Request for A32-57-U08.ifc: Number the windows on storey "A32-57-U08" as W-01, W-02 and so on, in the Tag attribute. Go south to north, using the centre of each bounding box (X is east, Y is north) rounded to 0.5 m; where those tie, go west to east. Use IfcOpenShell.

First a look at what the model holds.

```python
import ifcopenshell
import ifcopenshell.util.element
import ifcopenshell.util.placement

model = ifcopenshell.open("A32-57-U08.ifc")
print(model.schema)
storey = next(s for s in model.by_type("IfcBuildingStorey") if s.Name == "A32-57-U08")
windows = [e for e in ifcopenshell.util.element.get_decomposition(storey) if e.is_a("IfcWindow")]
for e in sorted(windows, key=lambda e: e.id()):
    origin = ifcopenshell.util.placement.get_local_placement(e.ObjectPlacement)[:3, 3]
    print(e.id(), e.Tag, e.Name, origin.round(2) + 0.0, sep=" | ")
```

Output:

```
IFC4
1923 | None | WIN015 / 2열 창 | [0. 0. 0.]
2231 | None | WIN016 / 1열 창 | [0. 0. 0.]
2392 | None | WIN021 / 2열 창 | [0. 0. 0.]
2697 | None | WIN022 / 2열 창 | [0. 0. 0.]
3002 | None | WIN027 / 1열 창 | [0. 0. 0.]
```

```python
import ifcopenshell
import ifcopenshell.geom
import ifcopenshell.util.element
import ifcopenshell.util.shape

model = ifcopenshell.open("A32-57-U08.ifc")
settings = ifcopenshell.geom.settings()
settings.set("use-world-coords", True)


def centre(element):
    shape = ifcopenshell.geom.create_shape(settings, element)
    return ifcopenshell.util.shape.get_bbox_centroid(shape.geometry)


storey = next(s for s in model.by_type("IfcBuildingStorey") if s.Name == "A32-57-U08")
windows = [e for e in ifcopenshell.util.element.get_decomposition(storey) if e.is_a("IfcWindow")]

# Insertion points can sit at a corner or the storey origin, so sort by the geometry (in metres).
centres = {e: centre(e) for e in windows}
windows.sort(key=lambda e: (round(centres[e][1] / 0.5), centres[e][0]))

for i, e in enumerate(windows, start=1):
    number = f"W-{i:02d}"
    e.Tag = number
    print(e.id(), number)

model.write("A32-57-U08_rev.ifc")
```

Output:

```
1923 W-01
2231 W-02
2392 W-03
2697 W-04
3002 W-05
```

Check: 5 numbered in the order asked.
